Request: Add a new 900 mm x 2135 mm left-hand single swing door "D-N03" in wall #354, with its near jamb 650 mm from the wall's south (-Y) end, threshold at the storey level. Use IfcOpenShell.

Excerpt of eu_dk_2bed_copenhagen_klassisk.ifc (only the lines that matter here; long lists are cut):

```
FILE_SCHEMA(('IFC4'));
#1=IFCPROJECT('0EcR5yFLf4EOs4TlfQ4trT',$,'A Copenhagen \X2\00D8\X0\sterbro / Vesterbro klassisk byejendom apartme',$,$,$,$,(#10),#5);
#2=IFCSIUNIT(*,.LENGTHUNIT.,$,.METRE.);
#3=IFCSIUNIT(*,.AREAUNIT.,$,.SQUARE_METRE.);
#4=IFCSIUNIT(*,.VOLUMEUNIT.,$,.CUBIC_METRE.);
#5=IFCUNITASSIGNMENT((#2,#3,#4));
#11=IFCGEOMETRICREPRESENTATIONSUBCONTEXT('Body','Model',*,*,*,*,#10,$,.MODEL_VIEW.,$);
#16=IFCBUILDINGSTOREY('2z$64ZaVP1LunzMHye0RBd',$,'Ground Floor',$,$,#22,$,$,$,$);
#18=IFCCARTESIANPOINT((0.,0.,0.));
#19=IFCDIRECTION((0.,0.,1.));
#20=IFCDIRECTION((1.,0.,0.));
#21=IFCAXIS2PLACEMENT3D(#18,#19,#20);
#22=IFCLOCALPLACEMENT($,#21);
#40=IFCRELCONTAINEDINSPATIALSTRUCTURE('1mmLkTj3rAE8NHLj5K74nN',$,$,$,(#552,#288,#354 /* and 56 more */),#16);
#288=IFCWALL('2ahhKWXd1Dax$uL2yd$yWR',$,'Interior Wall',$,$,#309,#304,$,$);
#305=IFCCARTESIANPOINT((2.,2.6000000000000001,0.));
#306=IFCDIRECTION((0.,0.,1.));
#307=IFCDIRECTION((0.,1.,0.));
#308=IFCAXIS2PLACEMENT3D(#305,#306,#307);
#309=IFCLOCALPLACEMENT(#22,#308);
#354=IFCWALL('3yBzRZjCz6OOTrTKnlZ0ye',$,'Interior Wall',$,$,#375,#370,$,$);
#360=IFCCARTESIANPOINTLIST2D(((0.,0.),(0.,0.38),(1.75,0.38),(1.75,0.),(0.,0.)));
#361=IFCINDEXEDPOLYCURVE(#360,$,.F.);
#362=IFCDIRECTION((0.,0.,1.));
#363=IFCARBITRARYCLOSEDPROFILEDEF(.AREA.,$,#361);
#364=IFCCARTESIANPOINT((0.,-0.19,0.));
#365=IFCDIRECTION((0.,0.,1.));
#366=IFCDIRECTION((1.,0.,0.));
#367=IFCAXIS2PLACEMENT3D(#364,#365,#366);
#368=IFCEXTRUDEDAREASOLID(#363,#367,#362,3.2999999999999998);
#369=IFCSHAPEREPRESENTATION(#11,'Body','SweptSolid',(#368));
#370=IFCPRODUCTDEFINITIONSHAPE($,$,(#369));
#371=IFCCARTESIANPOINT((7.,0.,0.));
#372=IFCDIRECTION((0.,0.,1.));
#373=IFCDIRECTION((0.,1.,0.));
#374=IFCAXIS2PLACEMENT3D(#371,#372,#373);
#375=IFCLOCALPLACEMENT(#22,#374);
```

```python
import numpy as np
import ifcopenshell
import ifcopenshell.api.feature
import ifcopenshell.api.geometry
import ifcopenshell.api.root
import ifcopenshell.api.spatial
import ifcopenshell.geom
import ifcopenshell.util.element
import ifcopenshell.util.placement
import ifcopenshell.util.representation
import ifcopenshell.util.shape
import ifcopenshell.util.unit

model = ifcopenshell.open("eu_dk_2bed_copenhagen_klassisk.ifc")
unit_scale = ifcopenshell.util.unit.calculate_unit_scale(model)
settings = ifcopenshell.geom.settings()


def volume(element):
    """Net volume in cubic metres, openings subtracted."""
    shape = ifcopenshell.geom.create_shape(settings, element)
    return ifcopenshell.util.shape.get_volume(shape.geometry)


wall = model.by_guid("3yBzRZjCz6OOTrTKnlZ0ye")
storey = ifcopenshell.util.element.get_container(wall, ifc_class="IfcBuildingStorey")
context = ifcopenshell.util.representation.get_context(model, "Model", "Body", "MODEL_VIEW")
before = volume(wall)

width, height, from_end, sill = 0.9, 2.135, 0.65, 0.0  # metres

# The wall runs along its own X axis, and the end named is its -X end.
wall_shape = ifcopenshell.geom.create_shape(settings, wall)
x, y, z = ifcopenshell.util.shape.get_vertices(wall_shape.geometry).T
start = x.min() + from_end
face, thickness = float(y.min()), float(y.max() - y.min())
wall_matrix = ifcopenshell.util.placement.get_local_placement(wall.ObjectPlacement)
level = ifcopenshell.util.placement.get_local_placement(storey.ObjectPlacement)[2, 3]


def in_wall(x, y):
    """Placement at x, y metres in the wall's axes, at sill height."""
    matrix = wall_matrix.copy()
    matrix[:, 3] = wall_matrix @ np.array([x / unit_scale, y / unit_scale, 0.0, 1.0])
    matrix[2, 3] = level + sill / unit_scale
    return matrix


# Opening: a box that overshoots both wall faces by 50 mm.
opening = ifcopenshell.api.root.create_entity(model, ifc_class="IfcOpeningElement", predefined_type="OPENING")
box = ifcopenshell.api.geometry.add_wall_representation(
    model, context=context, length=width, height=height, thickness=thickness + 0.1
)
ifcopenshell.api.geometry.assign_representation(model, product=opening, representation=box)
ifcopenshell.api.geometry.edit_object_placement(model, product=opening, matrix=in_wall(start, face - 0.05), is_si=False)
ifcopenshell.api.feature.add_feature(model, feature=opening, element=wall)

door = ifcopenshell.api.root.create_entity(model, ifc_class="IfcDoor", name="D-N03", predefined_type="DOOR")
door.OverallWidth, door.OverallHeight = width / unit_scale, height / unit_scale
door.OperationType = "SINGLE_SWING_LEFT"
body = ifcopenshell.api.geometry.add_door_representation(
    model,
    context=context,
    overall_width=door.OverallWidth,
    overall_height=door.OverallHeight,
    operation_type="SINGLE_SWING_LEFT",
    lining_properties={"LiningDepth": thickness / unit_scale, "ThresholdDepth": thickness / unit_scale},
)
ifcopenshell.api.geometry.assign_representation(model, product=door, representation=body)
ifcopenshell.api.spatial.assign_container(model, products=[door], relating_structure=storey)
ifcopenshell.api.feature.add_filling(model, opening=opening, element=door)

# The lining spans the wall, so the door starts at the wall face.
ifcopenshell.api.geometry.edit_object_placement(model, product=door, matrix=in_wall(start, face), is_si=False)

after = volume(wall)

print(f"wall volume {before:.3f} -> {after:.3f} m3")

model.write("eu_dk_2bed_copenhagen_klassisk_edited.ifc")
```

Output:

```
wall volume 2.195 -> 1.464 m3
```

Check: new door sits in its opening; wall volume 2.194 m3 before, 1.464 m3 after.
